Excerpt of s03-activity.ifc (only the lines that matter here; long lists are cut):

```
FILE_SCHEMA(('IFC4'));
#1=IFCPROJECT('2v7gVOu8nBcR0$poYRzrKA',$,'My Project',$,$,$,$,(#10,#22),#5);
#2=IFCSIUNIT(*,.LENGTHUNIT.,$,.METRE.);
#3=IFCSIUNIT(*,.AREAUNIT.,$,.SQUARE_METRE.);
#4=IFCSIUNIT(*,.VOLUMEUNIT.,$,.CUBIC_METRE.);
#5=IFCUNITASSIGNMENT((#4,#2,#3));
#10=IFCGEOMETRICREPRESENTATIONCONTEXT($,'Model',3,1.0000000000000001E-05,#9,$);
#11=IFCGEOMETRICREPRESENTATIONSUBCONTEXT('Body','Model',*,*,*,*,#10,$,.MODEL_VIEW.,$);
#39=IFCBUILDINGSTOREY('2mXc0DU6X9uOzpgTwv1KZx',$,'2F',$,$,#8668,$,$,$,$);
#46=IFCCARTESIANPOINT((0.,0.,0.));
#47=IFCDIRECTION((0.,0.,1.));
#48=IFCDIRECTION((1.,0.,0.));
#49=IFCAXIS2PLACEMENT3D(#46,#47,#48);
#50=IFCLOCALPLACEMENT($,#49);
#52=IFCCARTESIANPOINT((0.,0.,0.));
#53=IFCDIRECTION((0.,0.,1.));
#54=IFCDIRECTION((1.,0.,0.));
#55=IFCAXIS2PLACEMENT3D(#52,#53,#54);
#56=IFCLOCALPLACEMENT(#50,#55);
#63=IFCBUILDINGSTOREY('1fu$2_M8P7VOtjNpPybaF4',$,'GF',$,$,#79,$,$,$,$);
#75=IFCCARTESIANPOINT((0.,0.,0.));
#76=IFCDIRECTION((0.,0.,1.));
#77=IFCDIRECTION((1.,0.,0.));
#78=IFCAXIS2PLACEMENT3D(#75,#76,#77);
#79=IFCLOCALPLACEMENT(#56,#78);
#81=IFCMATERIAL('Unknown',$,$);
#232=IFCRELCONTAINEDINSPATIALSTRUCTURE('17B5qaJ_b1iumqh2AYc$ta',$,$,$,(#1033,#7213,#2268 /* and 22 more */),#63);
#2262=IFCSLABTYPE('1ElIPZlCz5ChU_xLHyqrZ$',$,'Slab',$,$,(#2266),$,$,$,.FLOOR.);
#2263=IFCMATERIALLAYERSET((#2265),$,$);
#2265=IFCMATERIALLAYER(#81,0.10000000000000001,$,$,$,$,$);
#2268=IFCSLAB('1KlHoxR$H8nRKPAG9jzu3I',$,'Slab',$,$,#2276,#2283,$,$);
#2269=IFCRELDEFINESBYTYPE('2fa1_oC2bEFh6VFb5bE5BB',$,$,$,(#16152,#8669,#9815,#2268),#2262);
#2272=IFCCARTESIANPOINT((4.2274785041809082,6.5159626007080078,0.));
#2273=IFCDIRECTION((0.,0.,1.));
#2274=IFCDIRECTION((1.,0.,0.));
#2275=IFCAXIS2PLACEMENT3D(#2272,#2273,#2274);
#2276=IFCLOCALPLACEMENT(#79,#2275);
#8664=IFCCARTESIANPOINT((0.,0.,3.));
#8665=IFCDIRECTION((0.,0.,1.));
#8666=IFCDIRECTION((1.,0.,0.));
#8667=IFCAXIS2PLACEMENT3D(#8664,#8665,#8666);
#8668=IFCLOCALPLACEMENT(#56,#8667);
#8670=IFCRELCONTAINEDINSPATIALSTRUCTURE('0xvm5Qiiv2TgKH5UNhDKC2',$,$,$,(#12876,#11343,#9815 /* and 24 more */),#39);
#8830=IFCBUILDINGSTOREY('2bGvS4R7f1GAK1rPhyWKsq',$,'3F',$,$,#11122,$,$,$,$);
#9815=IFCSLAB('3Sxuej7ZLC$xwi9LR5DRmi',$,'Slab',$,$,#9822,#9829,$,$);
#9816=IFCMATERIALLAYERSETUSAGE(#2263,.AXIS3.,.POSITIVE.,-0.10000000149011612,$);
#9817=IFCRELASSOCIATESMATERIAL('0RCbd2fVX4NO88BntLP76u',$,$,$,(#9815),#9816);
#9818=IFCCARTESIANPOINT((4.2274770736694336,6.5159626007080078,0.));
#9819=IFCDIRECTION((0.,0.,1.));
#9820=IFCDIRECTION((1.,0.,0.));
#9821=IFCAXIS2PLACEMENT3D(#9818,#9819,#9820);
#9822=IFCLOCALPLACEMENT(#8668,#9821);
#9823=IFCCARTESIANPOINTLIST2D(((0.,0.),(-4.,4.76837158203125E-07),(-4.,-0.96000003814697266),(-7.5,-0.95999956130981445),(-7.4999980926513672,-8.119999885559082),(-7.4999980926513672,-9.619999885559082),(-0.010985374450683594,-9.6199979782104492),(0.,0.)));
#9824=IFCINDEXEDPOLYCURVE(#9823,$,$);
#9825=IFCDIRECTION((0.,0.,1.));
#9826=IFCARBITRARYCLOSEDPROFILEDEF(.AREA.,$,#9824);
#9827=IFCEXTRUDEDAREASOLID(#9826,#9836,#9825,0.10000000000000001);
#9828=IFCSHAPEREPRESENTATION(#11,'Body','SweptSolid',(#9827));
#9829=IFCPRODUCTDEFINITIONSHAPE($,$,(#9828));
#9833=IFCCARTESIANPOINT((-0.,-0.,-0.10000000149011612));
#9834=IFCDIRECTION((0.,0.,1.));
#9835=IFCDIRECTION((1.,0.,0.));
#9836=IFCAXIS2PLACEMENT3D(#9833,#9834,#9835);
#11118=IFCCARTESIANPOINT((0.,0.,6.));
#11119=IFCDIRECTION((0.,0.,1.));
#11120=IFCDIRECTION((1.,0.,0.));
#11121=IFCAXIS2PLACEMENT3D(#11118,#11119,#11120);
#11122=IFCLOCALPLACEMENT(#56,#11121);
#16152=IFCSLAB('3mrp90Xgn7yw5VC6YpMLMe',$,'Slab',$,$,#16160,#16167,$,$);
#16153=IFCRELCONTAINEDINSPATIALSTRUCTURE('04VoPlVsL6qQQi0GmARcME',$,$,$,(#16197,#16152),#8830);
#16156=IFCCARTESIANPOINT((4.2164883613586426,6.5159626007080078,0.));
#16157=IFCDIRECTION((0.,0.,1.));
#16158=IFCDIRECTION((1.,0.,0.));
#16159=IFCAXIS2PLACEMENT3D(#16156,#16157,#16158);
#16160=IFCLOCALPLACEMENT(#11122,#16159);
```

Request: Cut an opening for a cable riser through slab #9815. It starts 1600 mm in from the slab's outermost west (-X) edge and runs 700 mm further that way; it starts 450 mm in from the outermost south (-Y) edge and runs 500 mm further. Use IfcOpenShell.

```python
import numpy as np
import ifcopenshell
import ifcopenshell.api.feature
import ifcopenshell.api.geometry
import ifcopenshell.api.root
import ifcopenshell.geom
import ifcopenshell.util.placement
import ifcopenshell.util.representation
import ifcopenshell.util.shape
import ifcopenshell.util.unit

model = ifcopenshell.open("s03-activity.ifc")
unit_scale = ifcopenshell.util.unit.calculate_unit_scale(model)
settings = ifcopenshell.geom.settings()


def volume(element):
    """Net volume in cubic metres, openings subtracted."""
    shape = ifcopenshell.geom.create_shape(settings, element)
    return ifcopenshell.util.shape.get_volume(shape.geometry)


slab = model.by_guid("3Sxuej7ZLC$xwi9LR5DRmi")
before = volume(slab)

# Extent in the slab's own axes, in metres. The edges named are its -X and -Y sides.
slab_shape = ifcopenshell.geom.create_shape(settings, slab)
vertices = ifcopenshell.util.shape.get_vertices(slab_shape.geometry)
x_min, y_min, bottom = vertices.min(axis=0)
top = vertices[:, 2].max()

opening = ifcopenshell.api.root.create_entity(model, ifc_class="IfcOpeningElement", name="Cable riser opening", predefined_type="OPENING")
context = ifcopenshell.util.representation.get_context(model, "Model", "Body", "MODEL_VIEW")
width, depth = 0.7, 0.5
outline = [(0.0, 0.0), (width, 0.0), (width, depth), (0.0, depth), (0.0, 0.0)]
# Overshoot both faces by 50 mm so the cut is clean.
shape = ifcopenshell.api.geometry.add_slab_representation(
    model, context=context, depth=top - bottom + 0.1, polyline=outline
)
ifcopenshell.api.geometry.assign_representation(model, product=opening, representation=shape)

matrix = ifcopenshell.util.placement.get_local_placement(slab.ObjectPlacement)
matrix[:, 3] = matrix @ np.append(np.array([x_min + 1.6, y_min + 0.45, bottom - 0.05]) / unit_scale, 1.0)
ifcopenshell.api.geometry.edit_object_placement(model, product=opening, matrix=matrix, is_si=False)
ifcopenshell.api.feature.add_feature(model, feature=opening, element=slab)

after = volume(slab)

print(f"slab volume {before:.3f} -> {after:.3f} m3")

model.write("s03-activity_edited.ifc")
```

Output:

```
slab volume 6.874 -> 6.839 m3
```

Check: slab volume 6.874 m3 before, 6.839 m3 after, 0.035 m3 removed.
